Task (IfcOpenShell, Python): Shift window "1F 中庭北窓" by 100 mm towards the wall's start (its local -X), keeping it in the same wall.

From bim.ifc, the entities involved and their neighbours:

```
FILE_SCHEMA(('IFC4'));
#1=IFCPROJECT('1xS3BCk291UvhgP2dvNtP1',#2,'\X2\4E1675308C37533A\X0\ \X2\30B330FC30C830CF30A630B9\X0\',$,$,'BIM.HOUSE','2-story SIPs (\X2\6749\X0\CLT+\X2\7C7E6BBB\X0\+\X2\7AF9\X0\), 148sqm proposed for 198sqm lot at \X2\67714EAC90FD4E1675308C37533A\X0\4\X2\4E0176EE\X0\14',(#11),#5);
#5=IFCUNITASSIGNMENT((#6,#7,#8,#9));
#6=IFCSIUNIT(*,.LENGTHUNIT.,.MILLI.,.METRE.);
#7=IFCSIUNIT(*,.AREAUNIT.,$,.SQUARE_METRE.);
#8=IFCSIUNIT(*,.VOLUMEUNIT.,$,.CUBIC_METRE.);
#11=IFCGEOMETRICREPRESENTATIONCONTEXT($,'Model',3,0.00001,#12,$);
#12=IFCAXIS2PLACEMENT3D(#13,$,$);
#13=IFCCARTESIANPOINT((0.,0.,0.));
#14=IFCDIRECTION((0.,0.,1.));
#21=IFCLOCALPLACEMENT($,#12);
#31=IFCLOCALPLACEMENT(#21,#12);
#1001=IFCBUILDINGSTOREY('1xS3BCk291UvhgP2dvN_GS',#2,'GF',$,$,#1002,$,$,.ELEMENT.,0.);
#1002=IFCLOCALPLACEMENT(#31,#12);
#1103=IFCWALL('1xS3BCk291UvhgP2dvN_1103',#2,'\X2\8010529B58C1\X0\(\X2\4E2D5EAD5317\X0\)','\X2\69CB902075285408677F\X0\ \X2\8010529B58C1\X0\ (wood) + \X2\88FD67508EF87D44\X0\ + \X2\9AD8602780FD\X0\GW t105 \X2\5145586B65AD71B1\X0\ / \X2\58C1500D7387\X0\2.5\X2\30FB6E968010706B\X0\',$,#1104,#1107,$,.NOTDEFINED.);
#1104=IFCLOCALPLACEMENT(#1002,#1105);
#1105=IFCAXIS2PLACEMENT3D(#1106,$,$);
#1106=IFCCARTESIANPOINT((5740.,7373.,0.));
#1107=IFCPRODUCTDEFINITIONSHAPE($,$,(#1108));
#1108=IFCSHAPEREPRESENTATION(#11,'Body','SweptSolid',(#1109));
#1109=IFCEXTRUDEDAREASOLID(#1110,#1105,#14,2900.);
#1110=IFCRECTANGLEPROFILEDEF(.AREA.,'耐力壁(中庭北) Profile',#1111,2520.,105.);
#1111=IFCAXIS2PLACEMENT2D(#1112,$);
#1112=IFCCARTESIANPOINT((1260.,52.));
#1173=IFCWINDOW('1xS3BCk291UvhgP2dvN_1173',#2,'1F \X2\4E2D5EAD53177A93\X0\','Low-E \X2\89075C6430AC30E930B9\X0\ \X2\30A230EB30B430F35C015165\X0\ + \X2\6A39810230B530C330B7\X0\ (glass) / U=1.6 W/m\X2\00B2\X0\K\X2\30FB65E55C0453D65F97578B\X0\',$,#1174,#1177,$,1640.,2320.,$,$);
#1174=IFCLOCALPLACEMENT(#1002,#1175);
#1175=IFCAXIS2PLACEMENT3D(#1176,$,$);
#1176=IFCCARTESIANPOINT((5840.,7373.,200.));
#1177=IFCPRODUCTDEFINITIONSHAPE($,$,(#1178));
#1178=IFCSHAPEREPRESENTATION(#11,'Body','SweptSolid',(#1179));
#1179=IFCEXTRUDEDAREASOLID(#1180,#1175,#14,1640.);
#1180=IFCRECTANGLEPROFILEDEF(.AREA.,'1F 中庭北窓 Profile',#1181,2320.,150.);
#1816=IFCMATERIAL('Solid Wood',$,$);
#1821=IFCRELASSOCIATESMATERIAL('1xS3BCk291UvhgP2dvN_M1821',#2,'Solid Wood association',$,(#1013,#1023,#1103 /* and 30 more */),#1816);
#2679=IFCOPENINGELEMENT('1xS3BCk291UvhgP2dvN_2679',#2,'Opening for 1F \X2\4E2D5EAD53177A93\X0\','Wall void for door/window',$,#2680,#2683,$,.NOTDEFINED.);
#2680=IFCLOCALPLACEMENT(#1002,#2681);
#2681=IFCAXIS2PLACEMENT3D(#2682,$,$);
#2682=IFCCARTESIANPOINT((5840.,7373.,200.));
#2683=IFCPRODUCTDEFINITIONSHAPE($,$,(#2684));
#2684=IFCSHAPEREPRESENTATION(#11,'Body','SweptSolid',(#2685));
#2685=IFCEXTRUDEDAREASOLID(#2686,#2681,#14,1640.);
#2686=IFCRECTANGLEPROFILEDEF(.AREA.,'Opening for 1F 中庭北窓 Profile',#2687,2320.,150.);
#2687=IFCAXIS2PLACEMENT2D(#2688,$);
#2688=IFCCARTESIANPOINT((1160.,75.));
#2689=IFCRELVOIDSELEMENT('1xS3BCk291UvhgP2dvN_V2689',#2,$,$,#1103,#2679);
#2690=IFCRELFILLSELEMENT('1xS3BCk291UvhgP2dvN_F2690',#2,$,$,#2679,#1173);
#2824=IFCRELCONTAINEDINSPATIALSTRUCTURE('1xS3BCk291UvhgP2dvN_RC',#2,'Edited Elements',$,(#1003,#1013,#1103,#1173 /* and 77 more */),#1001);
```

```python
import ifcopenshell
import ifcopenshell.api.geometry
import ifcopenshell.util.placement

model = ifcopenshell.open("bim.ifc")

window = model.by_guid("1xS3BCk291UvhgP2dvN_1173")
opening = window.FillsVoids[0].RelatingOpeningElement
wall = opening.VoidsElements[0].RelatingBuildingElement

wall_matrix = ifcopenshell.util.placement.get_local_placement(wall.ObjectPlacement)
shift = wall_matrix[:3, 0] * -100.0
before = ifcopenshell.util.placement.get_local_placement(window.ObjectPlacement)[:3, 3].copy()

# The window is not placed relative to its opening, so move both.
for product in (opening, window):
    matrix = ifcopenshell.util.placement.get_local_placement(product.ObjectPlacement)
    matrix[:3, 3] += shift
    ifcopenshell.api.geometry.edit_object_placement(model, product=product, matrix=matrix, is_si=False)

after = ifcopenshell.util.placement.get_local_placement(window.ObjectPlacement)[:3, 3]
print("window moved by", (after - before).round(3) + 0.0)

model.write("bim_rev.ifc")
```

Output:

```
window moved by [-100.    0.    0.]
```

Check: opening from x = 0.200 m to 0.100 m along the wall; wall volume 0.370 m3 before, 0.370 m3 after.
